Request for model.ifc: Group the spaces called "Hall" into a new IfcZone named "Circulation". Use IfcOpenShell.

First a look at what the model holds.

```python
import ifcopenshell

model = ifcopenshell.open("model.ifc")
print(model.schema)
seen = {}
for space in model.by_type("IfcSpace"):
    seen[space.LongName] = seen.get(space.LongName, 0) + 1
for name, count in sorted(seen.items(), key=str):
    print(count, "x", name)
print("zones:", [z.Name for z in model.by_type("IfcZone")][:20])
```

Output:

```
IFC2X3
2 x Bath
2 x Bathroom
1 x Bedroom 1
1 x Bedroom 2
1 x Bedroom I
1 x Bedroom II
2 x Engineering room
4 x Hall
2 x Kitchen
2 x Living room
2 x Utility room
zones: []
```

```python
import ifcopenshell
import ifcopenshell.api.group
import ifcopenshell.api.root

model = ifcopenshell.open("model.ifc")

names = {"Hall"}
spaces = [s for s in model.by_type("IfcSpace") if s.LongName in names]

zone = ifcopenshell.api.root.create_entity(model, ifc_class="IfcZone", name="Circulation")
ifcopenshell.api.group.assign_group(model, products=spaces, group=zone)
print(len(spaces), "spaces in", zone.Name)

model.write("model_edited.ifc")
```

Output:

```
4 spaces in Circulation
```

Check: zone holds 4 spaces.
